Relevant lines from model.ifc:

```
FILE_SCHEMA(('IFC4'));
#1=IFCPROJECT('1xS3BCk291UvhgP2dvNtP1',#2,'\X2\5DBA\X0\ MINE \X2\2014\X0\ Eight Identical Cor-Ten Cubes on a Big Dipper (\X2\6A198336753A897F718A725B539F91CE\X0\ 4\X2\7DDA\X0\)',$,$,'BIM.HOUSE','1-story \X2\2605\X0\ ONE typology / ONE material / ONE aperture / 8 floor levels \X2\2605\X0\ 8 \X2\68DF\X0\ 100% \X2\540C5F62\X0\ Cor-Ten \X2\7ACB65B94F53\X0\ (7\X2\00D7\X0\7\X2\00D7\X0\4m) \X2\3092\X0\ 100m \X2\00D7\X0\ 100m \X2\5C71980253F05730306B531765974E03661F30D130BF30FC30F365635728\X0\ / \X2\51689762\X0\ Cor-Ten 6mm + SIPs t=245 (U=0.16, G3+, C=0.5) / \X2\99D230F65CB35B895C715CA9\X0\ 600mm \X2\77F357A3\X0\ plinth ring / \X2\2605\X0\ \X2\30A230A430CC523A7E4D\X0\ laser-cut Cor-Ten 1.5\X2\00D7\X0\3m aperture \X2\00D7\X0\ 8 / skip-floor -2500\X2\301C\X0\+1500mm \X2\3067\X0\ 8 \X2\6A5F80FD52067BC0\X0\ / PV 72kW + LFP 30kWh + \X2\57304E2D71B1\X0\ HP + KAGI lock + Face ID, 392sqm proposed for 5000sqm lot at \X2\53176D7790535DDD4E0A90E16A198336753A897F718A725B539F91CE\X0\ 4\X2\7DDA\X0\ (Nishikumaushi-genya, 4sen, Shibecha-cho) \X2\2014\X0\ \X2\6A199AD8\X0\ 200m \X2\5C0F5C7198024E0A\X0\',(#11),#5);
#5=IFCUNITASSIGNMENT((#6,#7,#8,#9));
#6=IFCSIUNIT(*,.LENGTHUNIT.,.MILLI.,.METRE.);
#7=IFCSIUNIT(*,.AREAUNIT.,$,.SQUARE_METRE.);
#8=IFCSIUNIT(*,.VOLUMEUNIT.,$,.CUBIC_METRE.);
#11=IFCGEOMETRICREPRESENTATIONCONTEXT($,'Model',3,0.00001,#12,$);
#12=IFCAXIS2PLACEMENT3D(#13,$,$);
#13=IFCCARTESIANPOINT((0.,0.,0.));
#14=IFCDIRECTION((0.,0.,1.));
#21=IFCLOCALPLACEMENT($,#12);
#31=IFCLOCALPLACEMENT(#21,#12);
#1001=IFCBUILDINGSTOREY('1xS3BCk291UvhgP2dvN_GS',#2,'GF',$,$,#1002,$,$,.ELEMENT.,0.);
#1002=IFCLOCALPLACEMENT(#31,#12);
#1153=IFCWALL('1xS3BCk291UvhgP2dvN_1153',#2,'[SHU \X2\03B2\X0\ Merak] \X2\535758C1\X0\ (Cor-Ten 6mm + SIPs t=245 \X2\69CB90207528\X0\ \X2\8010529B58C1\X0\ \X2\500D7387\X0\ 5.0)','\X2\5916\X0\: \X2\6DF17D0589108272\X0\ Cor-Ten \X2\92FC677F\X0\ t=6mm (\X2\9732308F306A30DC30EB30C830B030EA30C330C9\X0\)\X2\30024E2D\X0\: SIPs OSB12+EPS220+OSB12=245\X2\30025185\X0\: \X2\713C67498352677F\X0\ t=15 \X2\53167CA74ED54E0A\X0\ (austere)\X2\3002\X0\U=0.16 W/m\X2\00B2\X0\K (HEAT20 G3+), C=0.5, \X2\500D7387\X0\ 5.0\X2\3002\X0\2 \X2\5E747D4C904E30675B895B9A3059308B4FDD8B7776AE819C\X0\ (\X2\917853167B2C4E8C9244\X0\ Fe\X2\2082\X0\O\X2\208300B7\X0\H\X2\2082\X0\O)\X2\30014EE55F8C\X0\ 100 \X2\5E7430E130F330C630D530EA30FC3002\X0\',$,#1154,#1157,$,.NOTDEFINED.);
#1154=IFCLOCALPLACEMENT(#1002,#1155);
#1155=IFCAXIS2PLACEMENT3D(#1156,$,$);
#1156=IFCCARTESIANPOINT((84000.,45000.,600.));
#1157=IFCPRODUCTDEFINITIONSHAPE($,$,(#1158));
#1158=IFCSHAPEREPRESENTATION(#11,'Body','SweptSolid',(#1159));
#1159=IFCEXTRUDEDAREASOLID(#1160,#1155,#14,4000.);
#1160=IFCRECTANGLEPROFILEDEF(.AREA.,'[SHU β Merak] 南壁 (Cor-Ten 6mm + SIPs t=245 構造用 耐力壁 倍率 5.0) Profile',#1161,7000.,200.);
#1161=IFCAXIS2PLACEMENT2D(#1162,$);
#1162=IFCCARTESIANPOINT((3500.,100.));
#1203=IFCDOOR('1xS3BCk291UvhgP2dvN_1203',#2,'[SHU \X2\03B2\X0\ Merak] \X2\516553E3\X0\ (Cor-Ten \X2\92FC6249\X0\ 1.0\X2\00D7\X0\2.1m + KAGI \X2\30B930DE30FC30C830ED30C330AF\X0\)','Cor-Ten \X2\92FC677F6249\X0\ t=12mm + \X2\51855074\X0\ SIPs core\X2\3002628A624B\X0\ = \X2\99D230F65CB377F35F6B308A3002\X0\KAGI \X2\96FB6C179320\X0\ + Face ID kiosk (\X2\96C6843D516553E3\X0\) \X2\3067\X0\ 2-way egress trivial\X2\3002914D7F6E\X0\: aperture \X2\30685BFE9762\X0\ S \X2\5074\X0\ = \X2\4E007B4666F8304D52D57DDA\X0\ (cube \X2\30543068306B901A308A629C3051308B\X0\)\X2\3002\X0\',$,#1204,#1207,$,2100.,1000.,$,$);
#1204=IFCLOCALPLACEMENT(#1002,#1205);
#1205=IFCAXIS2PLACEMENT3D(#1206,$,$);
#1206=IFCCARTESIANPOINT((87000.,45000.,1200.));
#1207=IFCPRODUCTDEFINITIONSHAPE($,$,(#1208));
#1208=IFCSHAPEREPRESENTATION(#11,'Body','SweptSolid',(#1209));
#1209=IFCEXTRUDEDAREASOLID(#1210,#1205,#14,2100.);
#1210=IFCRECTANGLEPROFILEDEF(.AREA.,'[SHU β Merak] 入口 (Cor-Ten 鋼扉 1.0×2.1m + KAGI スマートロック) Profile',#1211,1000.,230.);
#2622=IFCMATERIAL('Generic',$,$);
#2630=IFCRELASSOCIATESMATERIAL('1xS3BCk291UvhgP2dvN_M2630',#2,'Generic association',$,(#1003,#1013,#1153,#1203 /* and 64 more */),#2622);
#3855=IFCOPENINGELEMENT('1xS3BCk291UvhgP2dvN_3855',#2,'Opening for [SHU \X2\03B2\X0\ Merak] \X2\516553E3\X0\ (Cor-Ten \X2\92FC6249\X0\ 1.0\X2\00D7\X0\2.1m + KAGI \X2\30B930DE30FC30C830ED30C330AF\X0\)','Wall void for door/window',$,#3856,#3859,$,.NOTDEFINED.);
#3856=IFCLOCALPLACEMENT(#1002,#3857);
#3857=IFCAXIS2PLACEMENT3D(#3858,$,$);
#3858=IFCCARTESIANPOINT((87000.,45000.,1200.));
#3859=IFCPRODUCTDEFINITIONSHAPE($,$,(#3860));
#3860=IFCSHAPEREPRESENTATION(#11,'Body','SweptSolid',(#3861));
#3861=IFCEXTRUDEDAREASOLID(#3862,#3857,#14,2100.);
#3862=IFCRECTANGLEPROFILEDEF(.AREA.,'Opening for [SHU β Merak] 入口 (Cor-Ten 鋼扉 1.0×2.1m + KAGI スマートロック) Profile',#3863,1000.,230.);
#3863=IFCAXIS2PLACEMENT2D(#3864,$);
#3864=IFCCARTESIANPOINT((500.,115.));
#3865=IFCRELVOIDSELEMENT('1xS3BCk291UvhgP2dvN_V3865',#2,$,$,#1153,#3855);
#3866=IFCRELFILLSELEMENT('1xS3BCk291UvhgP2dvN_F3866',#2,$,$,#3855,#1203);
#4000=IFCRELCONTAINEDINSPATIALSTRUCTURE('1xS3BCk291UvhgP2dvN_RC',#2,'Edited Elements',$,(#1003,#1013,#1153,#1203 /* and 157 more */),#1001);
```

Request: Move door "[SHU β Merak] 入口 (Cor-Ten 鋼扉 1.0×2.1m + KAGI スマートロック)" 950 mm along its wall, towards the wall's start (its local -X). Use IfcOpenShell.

```python
import ifcopenshell
import ifcopenshell.api.geometry
import ifcopenshell.util.placement
import ifcopenshell.util.unit

model = ifcopenshell.open("model.ifc")
unit_scale = ifcopenshell.util.unit.calculate_unit_scale(model)

door = model.by_id(1203)
opening = door.FillsVoids[0].RelatingOpeningElement
wall = opening.VoidsElements[0].RelatingBuildingElement

wall_matrix = ifcopenshell.util.placement.get_local_placement(wall.ObjectPlacement)
shift = wall_matrix[:3, 0] * -0.95 / unit_scale
before = ifcopenshell.util.placement.get_local_placement(door.ObjectPlacement)[:3, 3].copy()

# The door is not placed relative to its opening, so move both.
for product in (opening, door):
    matrix = ifcopenshell.util.placement.get_local_placement(product.ObjectPlacement)
    matrix[:3, 3] += shift
    ifcopenshell.api.geometry.edit_object_placement(model, product=product, matrix=matrix, is_si=False)

after = ifcopenshell.util.placement.get_local_placement(door.ObjectPlacement)[:3, 3]
print("door moved by", (after - before).round(3) + 0.0)

model.write("model_v2.ifc")
```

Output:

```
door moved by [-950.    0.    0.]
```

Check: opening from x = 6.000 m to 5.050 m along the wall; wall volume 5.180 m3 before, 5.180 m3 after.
